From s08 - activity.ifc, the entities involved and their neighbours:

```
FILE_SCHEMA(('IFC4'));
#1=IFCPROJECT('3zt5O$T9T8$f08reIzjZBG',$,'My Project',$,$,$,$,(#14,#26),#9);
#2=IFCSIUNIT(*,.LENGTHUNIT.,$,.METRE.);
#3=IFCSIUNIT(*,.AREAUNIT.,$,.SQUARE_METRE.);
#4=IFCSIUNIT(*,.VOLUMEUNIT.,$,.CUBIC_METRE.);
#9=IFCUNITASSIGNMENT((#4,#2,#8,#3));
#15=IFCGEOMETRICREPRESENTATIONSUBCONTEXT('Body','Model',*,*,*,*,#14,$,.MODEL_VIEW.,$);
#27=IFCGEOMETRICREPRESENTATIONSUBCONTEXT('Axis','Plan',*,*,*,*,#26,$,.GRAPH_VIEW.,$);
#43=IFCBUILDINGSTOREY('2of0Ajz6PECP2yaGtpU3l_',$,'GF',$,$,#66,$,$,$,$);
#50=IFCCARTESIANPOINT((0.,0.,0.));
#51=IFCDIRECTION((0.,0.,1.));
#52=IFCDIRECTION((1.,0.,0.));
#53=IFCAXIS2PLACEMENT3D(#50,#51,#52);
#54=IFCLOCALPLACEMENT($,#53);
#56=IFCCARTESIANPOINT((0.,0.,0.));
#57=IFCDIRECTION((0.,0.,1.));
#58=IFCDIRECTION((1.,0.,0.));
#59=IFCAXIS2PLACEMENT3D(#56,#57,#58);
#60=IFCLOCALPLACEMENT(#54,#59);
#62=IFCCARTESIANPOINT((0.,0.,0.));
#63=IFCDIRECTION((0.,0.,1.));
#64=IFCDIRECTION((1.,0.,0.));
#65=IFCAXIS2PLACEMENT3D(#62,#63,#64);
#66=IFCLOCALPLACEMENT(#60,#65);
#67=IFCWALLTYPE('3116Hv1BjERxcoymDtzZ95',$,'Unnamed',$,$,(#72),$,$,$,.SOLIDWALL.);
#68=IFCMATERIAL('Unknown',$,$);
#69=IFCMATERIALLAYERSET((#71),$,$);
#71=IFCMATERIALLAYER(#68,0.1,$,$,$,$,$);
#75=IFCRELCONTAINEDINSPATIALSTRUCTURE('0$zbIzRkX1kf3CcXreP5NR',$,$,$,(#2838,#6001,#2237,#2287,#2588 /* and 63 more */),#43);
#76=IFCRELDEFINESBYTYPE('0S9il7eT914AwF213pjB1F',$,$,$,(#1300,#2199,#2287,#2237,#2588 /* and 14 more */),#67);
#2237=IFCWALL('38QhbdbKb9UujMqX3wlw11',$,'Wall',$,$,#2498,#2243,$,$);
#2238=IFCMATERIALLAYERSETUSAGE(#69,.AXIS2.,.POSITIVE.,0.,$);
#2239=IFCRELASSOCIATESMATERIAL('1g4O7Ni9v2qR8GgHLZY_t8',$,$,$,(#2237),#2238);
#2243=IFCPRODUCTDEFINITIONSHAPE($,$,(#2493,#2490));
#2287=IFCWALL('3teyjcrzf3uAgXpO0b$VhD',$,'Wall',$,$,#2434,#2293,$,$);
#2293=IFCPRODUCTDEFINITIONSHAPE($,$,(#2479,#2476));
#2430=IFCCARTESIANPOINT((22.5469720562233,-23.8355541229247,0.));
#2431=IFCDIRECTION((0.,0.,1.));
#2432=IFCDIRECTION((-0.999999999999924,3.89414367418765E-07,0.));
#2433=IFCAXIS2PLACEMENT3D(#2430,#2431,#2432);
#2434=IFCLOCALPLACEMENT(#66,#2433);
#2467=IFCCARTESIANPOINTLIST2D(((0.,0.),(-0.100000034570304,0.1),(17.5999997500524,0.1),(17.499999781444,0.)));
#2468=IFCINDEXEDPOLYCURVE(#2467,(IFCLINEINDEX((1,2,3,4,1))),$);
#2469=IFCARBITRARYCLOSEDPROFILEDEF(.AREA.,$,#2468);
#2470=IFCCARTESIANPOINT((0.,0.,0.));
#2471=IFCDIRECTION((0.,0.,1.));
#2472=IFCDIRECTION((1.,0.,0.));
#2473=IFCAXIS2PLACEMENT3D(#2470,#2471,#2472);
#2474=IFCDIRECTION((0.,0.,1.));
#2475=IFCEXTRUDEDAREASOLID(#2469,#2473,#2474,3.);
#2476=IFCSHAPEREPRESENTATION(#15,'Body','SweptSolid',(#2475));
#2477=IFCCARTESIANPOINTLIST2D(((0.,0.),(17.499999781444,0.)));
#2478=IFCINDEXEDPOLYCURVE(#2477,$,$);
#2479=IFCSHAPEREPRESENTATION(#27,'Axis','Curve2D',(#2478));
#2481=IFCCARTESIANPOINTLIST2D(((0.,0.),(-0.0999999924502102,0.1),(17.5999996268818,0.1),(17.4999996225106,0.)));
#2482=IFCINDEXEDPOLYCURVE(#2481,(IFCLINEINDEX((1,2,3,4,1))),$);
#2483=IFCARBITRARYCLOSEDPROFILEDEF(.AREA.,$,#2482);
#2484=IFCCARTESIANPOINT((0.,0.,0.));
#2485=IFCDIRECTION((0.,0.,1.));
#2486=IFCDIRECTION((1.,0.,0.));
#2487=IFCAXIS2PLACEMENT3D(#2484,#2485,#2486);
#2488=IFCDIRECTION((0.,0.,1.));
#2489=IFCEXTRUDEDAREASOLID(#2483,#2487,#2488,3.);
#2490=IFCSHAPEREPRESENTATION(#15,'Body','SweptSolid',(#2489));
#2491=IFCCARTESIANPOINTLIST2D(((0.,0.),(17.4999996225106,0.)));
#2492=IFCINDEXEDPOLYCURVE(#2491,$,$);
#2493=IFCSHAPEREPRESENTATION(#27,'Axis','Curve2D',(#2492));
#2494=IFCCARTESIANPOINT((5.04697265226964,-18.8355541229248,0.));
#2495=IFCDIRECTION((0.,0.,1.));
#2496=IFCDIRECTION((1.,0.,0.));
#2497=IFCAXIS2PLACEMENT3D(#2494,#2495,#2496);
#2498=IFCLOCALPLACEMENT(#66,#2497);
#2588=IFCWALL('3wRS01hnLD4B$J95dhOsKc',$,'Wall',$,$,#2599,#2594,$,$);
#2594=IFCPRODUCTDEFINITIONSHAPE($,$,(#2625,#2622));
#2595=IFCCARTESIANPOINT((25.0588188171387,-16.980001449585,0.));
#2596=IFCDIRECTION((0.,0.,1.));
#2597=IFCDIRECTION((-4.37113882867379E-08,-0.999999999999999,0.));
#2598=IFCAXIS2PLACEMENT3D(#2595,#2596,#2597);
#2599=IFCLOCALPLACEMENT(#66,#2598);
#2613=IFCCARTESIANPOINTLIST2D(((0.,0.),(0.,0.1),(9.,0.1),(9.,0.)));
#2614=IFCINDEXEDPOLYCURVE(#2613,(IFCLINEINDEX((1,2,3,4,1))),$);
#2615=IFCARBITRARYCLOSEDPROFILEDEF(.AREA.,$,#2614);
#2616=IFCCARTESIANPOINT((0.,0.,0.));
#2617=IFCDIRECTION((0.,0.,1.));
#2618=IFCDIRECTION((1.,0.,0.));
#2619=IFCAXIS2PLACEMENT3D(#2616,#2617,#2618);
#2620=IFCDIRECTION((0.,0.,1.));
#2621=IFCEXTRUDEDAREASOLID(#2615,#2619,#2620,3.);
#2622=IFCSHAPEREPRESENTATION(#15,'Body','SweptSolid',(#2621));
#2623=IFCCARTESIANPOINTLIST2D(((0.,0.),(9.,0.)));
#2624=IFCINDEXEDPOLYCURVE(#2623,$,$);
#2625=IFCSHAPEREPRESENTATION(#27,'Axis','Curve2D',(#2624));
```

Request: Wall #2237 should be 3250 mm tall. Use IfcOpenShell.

```python
import ifcopenshell
import ifcopenshell.geom
import ifcopenshell.util.representation
import ifcopenshell.util.shape
import ifcopenshell.util.unit

model = ifcopenshell.open("s08 - activity.ifc")
unit_scale = ifcopenshell.util.unit.calculate_unit_scale(model)
settings = ifcopenshell.geom.settings()


def volume(element):
    """Net volume in cubic metres, openings subtracted."""
    shape = ifcopenshell.geom.create_shape(settings, element)
    return ifcopenshell.util.shape.get_volume(shape.geometry)


wall = model.by_guid("38QhbdbKb9UujMqX3wlw11")
before = volume(wall)

body = ifcopenshell.util.representation.get_representation(wall, "Model", "Body")
solid = body.Items[0]
old_height = solid.Depth
solid.Depth = 3.25 / unit_scale
after = volume(wall)

print(f"height {old_height:g} -> {solid.Depth:g}, volume {before:.3f} -> {after:.3f} m3")

model.write("s08 - activity_edited.ifc")
```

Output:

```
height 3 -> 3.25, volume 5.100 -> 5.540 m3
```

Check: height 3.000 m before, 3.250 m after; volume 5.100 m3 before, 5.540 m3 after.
